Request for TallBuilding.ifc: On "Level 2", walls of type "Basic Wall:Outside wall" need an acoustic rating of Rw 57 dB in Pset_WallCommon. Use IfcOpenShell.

First a look at what the model holds.

```python
import ifcopenshell
import ifcopenshell.util.element

model = ifcopenshell.open("TallBuilding.ifc")
print(model.schema)
storey = next(s for s in model.by_type("IfcBuildingStorey") if s.Name == "Level 2")
walls = [e for e in ifcopenshell.util.element.get_decomposition(storey) if e.is_a("IfcWall")]
seen = {}
for e in walls:
    element_type = ifcopenshell.util.element.get_type(e)
    key = (element_type.Name if element_type != e and element_type else None, ifcopenshell.util.element.get_pset(e, "Pset_WallCommon", "AcousticRating"))
    seen[key] = seen.get(key, 0) + 1
for (name, value), count in sorted(seen.items(), key=str):
    print(count, "x", name, "|", value)
```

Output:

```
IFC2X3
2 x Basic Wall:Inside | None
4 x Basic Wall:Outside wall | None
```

```python
import ifcopenshell
import ifcopenshell.api.pset
import ifcopenshell.util.element

model = ifcopenshell.open("TallBuilding.ifc")

storey = next(s for s in model.by_type("IfcBuildingStorey") if s.Name == "Level 2")
walls = [e for e in ifcopenshell.util.element.get_decomposition(storey) if e.is_a("IfcWall")]

count = 0
for e in walls:
    element_type = ifcopenshell.util.element.get_type(e)
    if element_type in (None, e) or element_type.Name != "Basic Wall:Outside wall":
        continue
    # add_pset returns the element's existing set when there is one.
    pset = ifcopenshell.api.pset.add_pset(model, product=e, name="Pset_WallCommon")
    ifcopenshell.api.pset.edit_pset(model, pset=pset, properties={"AcousticRating": "Rw 57 dB"})
    count += 1

print(count, "walls updated")

model.write("TallBuilding_edited.ifc")
```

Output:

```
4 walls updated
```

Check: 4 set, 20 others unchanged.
